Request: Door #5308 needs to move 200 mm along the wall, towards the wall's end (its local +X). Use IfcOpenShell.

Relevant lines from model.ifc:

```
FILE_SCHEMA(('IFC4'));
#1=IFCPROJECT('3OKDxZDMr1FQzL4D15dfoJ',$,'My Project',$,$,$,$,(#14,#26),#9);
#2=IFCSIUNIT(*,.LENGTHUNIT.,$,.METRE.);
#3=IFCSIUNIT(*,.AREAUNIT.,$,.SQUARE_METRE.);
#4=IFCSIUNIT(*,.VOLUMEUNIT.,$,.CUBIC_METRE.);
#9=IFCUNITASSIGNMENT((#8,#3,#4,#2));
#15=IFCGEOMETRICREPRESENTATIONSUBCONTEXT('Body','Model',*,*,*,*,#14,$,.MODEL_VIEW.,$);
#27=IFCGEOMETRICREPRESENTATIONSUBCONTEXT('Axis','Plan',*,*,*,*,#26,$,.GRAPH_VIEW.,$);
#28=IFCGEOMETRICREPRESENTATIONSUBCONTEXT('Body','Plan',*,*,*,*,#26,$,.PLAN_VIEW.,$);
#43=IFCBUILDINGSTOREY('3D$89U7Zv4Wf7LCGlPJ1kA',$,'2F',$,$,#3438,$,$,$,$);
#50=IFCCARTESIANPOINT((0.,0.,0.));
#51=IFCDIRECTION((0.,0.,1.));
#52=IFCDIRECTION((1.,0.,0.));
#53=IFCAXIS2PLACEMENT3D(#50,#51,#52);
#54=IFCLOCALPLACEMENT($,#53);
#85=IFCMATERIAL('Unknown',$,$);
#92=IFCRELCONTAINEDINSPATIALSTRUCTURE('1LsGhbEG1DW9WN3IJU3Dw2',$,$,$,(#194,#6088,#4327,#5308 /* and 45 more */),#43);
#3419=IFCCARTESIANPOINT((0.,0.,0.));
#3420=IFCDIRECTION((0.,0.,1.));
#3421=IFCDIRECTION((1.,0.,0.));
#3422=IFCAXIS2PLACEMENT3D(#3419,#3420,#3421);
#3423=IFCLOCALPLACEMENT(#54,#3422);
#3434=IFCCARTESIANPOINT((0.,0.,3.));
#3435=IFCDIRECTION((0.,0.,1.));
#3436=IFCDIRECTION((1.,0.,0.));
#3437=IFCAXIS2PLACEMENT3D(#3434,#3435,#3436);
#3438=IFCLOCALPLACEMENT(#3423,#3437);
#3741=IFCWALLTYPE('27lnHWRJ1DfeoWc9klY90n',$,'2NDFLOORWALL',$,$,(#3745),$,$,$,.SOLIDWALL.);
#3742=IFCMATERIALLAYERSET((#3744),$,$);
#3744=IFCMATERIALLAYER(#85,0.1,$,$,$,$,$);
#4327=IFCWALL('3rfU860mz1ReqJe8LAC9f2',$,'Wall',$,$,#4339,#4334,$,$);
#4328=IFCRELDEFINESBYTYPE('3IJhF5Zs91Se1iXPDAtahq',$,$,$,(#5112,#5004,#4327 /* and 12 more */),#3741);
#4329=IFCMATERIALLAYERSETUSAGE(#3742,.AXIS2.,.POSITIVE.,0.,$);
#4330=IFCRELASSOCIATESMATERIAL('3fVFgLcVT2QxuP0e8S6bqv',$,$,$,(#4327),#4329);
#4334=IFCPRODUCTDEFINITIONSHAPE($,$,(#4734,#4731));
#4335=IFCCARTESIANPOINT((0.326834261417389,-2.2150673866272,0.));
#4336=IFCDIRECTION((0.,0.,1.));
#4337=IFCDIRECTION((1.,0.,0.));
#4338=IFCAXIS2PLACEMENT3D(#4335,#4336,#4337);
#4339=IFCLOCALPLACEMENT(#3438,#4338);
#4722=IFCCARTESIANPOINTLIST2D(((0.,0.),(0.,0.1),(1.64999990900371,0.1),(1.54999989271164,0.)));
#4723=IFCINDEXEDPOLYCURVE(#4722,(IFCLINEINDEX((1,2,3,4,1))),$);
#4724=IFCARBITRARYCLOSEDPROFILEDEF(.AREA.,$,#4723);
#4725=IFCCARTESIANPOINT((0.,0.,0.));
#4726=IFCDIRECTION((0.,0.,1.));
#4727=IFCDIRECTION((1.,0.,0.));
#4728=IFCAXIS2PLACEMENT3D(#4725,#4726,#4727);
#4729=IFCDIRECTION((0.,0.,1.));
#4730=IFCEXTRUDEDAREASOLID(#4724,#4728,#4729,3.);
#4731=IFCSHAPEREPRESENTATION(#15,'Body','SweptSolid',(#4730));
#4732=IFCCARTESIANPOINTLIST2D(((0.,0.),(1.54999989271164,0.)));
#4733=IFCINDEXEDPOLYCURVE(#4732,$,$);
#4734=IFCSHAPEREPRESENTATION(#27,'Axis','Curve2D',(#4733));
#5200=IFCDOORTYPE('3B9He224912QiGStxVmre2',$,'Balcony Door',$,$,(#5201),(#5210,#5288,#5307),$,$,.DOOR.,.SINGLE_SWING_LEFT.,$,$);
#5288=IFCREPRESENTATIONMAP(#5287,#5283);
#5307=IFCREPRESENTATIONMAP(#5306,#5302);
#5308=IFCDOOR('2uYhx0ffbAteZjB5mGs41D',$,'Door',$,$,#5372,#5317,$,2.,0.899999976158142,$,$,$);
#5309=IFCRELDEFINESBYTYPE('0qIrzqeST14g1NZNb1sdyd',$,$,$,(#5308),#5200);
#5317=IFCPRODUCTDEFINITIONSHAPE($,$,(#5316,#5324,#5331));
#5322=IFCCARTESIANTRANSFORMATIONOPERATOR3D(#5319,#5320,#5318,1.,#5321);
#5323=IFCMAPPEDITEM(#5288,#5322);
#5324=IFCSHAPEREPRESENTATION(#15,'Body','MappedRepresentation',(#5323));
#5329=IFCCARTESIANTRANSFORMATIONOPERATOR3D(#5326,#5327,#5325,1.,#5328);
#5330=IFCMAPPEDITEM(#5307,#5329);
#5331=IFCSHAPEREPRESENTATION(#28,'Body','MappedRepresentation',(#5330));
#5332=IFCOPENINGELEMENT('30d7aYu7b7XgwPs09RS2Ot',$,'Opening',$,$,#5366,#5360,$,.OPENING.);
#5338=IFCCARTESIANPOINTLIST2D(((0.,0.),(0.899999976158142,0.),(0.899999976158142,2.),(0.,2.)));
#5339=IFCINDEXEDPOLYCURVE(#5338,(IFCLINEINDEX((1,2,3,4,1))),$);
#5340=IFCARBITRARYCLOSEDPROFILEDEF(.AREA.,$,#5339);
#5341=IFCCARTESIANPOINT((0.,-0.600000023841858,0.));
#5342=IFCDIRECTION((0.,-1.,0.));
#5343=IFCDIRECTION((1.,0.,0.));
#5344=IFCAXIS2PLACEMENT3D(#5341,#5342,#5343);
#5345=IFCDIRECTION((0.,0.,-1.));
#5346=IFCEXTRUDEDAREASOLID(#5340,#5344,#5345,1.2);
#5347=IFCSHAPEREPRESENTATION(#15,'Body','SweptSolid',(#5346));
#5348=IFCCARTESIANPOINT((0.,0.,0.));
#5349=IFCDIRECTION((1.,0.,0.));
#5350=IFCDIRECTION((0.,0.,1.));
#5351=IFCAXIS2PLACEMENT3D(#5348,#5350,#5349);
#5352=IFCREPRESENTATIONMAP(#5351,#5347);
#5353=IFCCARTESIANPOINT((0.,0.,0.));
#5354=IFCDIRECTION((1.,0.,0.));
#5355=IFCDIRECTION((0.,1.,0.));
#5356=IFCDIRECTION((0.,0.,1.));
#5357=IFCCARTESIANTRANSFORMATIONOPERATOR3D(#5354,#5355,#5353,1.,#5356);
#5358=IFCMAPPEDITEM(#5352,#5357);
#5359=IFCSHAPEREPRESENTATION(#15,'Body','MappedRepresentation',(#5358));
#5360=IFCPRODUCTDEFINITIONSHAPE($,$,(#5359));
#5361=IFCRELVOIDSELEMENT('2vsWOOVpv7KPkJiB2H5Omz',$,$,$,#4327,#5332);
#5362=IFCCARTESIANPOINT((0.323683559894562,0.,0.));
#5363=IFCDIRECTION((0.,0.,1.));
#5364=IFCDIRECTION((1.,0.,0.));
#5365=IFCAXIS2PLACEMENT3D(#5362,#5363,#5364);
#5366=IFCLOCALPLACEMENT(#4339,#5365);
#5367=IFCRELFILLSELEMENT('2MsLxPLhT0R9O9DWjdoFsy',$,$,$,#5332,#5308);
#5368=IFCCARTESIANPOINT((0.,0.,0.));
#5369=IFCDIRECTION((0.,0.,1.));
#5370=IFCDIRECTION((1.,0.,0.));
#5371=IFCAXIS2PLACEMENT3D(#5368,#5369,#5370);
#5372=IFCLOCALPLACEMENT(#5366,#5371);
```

```python
import ifcopenshell
import ifcopenshell.api.geometry
import ifcopenshell.util.placement

model = ifcopenshell.open("model.ifc")

door = model.by_id(5308)
opening = door.FillsVoids[0].RelatingOpeningElement
wall = opening.VoidsElements[0].RelatingBuildingElement

wall_matrix = ifcopenshell.util.placement.get_local_placement(wall.ObjectPlacement)
shift = wall_matrix[:3, 0] * 0.2
before = ifcopenshell.util.placement.get_local_placement(door.ObjectPlacement)[:3, 3].copy()

# The door is placed relative to its opening, so it follows when the opening moves.
matrix = ifcopenshell.util.placement.get_local_placement(opening.ObjectPlacement)
matrix[:3, 3] += shift
ifcopenshell.api.geometry.edit_object_placement(
    model, product=opening, matrix=matrix, is_si=False, should_transform_children=True
)

after = ifcopenshell.util.placement.get_local_placement(door.ObjectPlacement)[:3, 3]
print("door moved by", (after - before).round(3) + 0.0)

model.write("model_edited.ifc")
```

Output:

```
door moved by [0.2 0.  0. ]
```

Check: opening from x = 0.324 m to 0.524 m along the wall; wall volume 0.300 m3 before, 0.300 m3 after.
